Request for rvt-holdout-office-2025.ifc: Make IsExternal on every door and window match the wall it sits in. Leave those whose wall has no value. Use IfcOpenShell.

First a look at what the model holds.

```python
import ifcopenshell
import ifcopenshell.util.element

model = ifcopenshell.open("rvt-holdout-office-2025.ifc")
print(model.schema)
seen = {}
for e in model.by_type("IfcDoor") + model.by_type("IfcWindow"):
    if not e.FillsVoids:
        continue
    host = e.FillsVoids[0].RelatingOpeningElement.VoidsElements[0].RelatingBuildingElement
    own = ifcopenshell.util.element.get_pset(e, f"Pset_{e.is_a()[3:].removesuffix('StandardCase')}Common", "IsExternal")
    wall = ifcopenshell.util.element.get_pset(host, "Pset_WallCommon", "IsExternal")
    seen[e.is_a(), own, wall] = seen.get((e.is_a(), own, wall), 0) + 1
for (cls, own, wall), count in sorted(seen.items(), key=str):
    print(count, cls, "IsExternal:", own, "| host wall:", wall)
```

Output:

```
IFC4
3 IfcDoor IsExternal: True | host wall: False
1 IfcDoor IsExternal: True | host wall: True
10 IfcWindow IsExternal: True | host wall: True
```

```python
import ifcopenshell
import ifcopenshell.api.pset
import ifcopenshell.util.element

model = ifcopenshell.open("rvt-holdout-office-2025.ifc")

count = 0
for ifc_class, pset_name in (("IfcDoor", "Pset_DoorCommon"), ("IfcWindow", "Pset_WindowCommon")):
    for e in model.by_type(ifc_class):
        if not e.FillsVoids:
            continue
        host = e.FillsVoids[0].RelatingOpeningElement.VoidsElements[0].RelatingBuildingElement
        external = ifcopenshell.util.element.get_pset(host, "Pset_WallCommon", "IsExternal")
        if external is None or ifcopenshell.util.element.get_pset(e, pset_name, "IsExternal") == external:
            continue
        pset = ifcopenshell.api.pset.add_pset(model, product=e, name=pset_name)
        ifcopenshell.api.pset.edit_pset(model, pset=pset, properties={"IsExternal": external})
        count += 1

print(count, "updated")

model.write("rvt-holdout-office-2025_edited.ifc")
```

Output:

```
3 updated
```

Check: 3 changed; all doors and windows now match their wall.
